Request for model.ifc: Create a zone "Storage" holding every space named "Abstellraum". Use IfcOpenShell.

First a look at what the model holds.

```python
import ifcopenshell

model = ifcopenshell.open("model.ifc")
print(model.schema)
seen = {}
for space in model.by_type("IfcSpace"):
    seen[space.LongName] = seen.get(space.LongName, 0) + 1
for name, count in sorted(seen.items(), key=str):
    print(count, "x", name)
print("zones:", [z.Name for z in model.by_type("IfcZone")][:20])
```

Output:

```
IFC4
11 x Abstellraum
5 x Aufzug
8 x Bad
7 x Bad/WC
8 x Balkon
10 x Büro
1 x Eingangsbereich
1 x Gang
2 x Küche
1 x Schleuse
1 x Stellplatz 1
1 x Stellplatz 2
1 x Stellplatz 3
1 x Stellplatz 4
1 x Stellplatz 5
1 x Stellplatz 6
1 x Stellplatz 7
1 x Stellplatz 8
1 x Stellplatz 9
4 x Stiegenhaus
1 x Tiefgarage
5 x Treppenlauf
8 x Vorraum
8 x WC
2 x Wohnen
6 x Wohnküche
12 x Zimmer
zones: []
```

```python
import ifcopenshell
import ifcopenshell.api.group
import ifcopenshell.api.root

model = ifcopenshell.open("model.ifc")

names = {"Abstellraum"}
spaces = [s for s in model.by_type("IfcSpace") if s.LongName in names]

zone = ifcopenshell.api.root.create_entity(model, ifc_class="IfcZone", name="Storage")
ifcopenshell.api.group.assign_group(model, products=spaces, group=zone)
print(len(spaces), "spaces in", zone.Name)

model.write("model_rev.ifc")
```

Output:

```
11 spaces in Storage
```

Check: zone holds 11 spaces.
